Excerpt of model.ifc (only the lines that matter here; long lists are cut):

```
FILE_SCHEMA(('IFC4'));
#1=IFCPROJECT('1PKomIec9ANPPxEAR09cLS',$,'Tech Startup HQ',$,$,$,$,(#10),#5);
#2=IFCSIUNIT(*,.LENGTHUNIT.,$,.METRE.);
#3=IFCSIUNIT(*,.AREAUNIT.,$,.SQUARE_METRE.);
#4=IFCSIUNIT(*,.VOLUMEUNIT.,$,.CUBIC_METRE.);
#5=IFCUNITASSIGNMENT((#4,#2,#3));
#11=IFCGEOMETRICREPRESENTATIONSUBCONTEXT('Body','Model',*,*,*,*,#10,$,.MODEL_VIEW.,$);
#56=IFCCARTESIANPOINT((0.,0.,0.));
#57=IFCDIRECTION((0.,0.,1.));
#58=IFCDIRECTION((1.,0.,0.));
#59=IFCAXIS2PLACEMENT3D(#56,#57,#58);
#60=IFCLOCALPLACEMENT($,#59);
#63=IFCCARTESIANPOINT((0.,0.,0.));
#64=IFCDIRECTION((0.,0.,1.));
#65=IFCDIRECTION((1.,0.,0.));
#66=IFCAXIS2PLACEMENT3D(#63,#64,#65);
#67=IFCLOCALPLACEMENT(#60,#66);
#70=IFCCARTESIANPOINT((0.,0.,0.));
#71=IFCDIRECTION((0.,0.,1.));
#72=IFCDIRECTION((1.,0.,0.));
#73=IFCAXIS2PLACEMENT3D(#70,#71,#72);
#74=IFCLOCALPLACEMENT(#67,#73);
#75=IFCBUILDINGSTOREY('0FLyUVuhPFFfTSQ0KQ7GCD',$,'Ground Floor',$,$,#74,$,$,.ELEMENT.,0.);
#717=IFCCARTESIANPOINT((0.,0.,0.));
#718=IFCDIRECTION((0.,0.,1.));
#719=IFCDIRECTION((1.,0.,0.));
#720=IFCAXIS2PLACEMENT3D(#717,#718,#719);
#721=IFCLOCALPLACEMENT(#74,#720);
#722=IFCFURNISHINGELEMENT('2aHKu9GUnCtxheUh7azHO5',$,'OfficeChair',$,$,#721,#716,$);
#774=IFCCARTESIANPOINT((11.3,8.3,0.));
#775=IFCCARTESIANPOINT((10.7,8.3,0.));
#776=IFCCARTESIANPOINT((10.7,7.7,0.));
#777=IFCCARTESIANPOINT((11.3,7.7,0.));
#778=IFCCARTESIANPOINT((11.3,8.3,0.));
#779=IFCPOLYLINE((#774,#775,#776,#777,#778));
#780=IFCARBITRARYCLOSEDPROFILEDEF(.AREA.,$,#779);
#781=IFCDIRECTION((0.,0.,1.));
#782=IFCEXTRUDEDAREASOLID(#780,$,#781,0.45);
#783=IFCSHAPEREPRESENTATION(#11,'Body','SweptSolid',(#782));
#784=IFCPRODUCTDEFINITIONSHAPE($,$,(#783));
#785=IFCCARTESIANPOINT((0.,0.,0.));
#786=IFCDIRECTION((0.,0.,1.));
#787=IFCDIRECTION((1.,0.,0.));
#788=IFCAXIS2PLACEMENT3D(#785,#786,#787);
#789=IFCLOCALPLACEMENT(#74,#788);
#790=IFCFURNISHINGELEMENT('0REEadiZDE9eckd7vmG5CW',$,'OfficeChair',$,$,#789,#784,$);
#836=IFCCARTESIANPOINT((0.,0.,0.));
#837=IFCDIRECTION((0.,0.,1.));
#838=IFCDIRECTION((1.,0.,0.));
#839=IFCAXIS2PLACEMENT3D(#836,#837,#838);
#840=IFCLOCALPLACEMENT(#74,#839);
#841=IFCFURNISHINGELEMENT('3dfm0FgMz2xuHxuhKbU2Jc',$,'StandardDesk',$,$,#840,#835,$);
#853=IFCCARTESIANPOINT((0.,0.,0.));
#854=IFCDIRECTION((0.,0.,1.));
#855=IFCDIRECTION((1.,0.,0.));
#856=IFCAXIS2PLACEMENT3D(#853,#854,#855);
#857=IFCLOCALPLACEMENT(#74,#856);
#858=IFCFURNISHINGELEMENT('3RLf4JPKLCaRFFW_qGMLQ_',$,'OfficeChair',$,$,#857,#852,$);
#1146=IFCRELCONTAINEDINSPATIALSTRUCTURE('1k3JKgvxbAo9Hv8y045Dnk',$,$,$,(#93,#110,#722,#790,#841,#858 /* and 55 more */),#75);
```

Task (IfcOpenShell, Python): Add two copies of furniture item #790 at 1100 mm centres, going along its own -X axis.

```python
import ifcopenshell
import ifcopenshell.api.geometry
import ifcopenshell.api.root
import ifcopenshell.util.element
import ifcopenshell.util.placement

model = ifcopenshell.open("model.ifc")

source = model.by_guid("0REEadiZDE9eckd7vmG5CW")
base = ifcopenshell.util.placement.get_local_placement(source.ObjectPlacement)
step = -base[:3, 0] * 1.1

for i in range(1, 3):
    copy = ifcopenshell.api.root.copy_class(model, product=source)
    copy.Representation = ifcopenshell.util.element.copy_deep(
        model, source.Representation, exclude=["IfcGeometricRepresentationContext", "IfcRepresentationMap"]
    )
    matrix = base.copy()
    matrix[:3, 3] += i * step
    print("added at", matrix[:3, 3].round(3) + 0.0)
    ifcopenshell.api.geometry.edit_object_placement(model, product=copy, matrix=matrix, is_si=False)

model.write("model_v2.ifc")
```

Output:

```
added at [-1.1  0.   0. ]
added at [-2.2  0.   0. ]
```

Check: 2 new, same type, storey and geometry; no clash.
